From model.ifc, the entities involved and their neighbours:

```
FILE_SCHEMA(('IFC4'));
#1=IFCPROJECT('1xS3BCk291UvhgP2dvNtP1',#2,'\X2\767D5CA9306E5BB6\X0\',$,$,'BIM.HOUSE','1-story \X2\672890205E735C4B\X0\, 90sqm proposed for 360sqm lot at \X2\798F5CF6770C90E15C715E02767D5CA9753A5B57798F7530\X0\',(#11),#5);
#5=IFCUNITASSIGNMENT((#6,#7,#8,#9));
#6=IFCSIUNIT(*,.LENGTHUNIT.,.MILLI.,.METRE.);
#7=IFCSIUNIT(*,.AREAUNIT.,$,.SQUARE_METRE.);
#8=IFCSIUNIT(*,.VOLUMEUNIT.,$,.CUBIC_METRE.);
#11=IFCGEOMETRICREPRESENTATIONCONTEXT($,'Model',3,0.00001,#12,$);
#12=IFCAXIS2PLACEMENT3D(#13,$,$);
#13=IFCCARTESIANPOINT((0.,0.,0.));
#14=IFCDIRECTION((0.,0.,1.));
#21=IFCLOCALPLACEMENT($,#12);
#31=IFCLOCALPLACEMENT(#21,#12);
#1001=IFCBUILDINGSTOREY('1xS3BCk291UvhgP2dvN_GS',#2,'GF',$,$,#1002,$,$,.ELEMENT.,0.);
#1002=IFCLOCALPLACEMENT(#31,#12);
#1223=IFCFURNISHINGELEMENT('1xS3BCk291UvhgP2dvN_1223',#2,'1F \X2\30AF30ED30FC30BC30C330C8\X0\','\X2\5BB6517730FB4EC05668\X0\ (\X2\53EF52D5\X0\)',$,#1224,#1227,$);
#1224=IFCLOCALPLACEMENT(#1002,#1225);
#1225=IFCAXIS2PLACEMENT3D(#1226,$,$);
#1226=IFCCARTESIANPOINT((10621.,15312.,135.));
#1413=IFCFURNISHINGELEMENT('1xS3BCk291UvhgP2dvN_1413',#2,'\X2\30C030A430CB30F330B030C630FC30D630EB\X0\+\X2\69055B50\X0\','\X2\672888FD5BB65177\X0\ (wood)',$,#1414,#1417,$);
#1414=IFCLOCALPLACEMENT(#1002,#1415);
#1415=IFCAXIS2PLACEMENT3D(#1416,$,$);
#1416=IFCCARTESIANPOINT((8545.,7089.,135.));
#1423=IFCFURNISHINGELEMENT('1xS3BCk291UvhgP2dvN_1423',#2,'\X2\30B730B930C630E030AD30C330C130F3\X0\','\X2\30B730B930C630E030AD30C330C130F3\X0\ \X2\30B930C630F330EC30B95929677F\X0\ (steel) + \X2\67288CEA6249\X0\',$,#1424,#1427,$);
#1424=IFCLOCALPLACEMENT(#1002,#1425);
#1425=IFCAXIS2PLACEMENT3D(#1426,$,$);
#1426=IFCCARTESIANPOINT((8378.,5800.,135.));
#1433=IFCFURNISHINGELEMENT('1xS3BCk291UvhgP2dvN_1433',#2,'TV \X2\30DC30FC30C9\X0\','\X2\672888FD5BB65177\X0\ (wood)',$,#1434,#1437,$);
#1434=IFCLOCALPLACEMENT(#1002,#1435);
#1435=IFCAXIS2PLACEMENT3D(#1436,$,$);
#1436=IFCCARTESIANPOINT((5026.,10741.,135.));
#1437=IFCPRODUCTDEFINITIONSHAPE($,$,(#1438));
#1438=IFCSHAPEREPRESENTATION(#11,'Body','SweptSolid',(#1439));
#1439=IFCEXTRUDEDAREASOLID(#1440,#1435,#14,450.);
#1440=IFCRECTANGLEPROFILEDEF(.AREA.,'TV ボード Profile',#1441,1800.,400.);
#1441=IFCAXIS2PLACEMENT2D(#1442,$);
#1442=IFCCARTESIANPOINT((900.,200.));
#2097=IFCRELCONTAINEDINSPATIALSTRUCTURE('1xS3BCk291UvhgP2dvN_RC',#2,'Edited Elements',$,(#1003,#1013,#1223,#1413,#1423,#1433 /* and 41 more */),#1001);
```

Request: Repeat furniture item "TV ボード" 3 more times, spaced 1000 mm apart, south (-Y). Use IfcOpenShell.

```python
import numpy as np
import ifcopenshell
import ifcopenshell.api.geometry
import ifcopenshell.api.root
import ifcopenshell.util.element
import ifcopenshell.util.placement
import ifcopenshell.util.unit

model = ifcopenshell.open("model.ifc")
unit_scale = ifcopenshell.util.unit.calculate_unit_scale(model)


def reuse_history(source, copy):
    """copy_class also copies each property set's owner history, people and application; keep the originals."""
    for rel in copy.IsDefinedBy:
        if rel.is_a("IfcRelDefinesByProperties") and (history := rel.RelatingPropertyDefinition.OwnerHistory):
            rel.RelatingPropertyDefinition.OwnerHistory = source.OwnerHistory
            ifcopenshell.util.element.remove_deep2(model, history)


source = model.by_guid("1xS3BCk291UvhgP2dvN_1433")
base = ifcopenshell.util.placement.get_local_placement(source.ObjectPlacement)
step = np.array([0.0, -1.0, 0.0]) * 1 / unit_scale

for i in range(1, 4):
    copy = ifcopenshell.api.root.copy_class(model, product=source)
    copy.Representation = ifcopenshell.util.element.copy_deep(
        model, source.Representation, exclude=["IfcGeometricRepresentationContext", "IfcRepresentationMap"]
    )
    reuse_history(source, copy)
    matrix = base.copy()
    matrix[:3, 3] += i * step
    print("added at", matrix[:3, 3].round(3) + 0.0)
    ifcopenshell.api.geometry.edit_object_placement(model, product=copy, matrix=matrix, is_si=False)

model.write("model_updated.ifc")
```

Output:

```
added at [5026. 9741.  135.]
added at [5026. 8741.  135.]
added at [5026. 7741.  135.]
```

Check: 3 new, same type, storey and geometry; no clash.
